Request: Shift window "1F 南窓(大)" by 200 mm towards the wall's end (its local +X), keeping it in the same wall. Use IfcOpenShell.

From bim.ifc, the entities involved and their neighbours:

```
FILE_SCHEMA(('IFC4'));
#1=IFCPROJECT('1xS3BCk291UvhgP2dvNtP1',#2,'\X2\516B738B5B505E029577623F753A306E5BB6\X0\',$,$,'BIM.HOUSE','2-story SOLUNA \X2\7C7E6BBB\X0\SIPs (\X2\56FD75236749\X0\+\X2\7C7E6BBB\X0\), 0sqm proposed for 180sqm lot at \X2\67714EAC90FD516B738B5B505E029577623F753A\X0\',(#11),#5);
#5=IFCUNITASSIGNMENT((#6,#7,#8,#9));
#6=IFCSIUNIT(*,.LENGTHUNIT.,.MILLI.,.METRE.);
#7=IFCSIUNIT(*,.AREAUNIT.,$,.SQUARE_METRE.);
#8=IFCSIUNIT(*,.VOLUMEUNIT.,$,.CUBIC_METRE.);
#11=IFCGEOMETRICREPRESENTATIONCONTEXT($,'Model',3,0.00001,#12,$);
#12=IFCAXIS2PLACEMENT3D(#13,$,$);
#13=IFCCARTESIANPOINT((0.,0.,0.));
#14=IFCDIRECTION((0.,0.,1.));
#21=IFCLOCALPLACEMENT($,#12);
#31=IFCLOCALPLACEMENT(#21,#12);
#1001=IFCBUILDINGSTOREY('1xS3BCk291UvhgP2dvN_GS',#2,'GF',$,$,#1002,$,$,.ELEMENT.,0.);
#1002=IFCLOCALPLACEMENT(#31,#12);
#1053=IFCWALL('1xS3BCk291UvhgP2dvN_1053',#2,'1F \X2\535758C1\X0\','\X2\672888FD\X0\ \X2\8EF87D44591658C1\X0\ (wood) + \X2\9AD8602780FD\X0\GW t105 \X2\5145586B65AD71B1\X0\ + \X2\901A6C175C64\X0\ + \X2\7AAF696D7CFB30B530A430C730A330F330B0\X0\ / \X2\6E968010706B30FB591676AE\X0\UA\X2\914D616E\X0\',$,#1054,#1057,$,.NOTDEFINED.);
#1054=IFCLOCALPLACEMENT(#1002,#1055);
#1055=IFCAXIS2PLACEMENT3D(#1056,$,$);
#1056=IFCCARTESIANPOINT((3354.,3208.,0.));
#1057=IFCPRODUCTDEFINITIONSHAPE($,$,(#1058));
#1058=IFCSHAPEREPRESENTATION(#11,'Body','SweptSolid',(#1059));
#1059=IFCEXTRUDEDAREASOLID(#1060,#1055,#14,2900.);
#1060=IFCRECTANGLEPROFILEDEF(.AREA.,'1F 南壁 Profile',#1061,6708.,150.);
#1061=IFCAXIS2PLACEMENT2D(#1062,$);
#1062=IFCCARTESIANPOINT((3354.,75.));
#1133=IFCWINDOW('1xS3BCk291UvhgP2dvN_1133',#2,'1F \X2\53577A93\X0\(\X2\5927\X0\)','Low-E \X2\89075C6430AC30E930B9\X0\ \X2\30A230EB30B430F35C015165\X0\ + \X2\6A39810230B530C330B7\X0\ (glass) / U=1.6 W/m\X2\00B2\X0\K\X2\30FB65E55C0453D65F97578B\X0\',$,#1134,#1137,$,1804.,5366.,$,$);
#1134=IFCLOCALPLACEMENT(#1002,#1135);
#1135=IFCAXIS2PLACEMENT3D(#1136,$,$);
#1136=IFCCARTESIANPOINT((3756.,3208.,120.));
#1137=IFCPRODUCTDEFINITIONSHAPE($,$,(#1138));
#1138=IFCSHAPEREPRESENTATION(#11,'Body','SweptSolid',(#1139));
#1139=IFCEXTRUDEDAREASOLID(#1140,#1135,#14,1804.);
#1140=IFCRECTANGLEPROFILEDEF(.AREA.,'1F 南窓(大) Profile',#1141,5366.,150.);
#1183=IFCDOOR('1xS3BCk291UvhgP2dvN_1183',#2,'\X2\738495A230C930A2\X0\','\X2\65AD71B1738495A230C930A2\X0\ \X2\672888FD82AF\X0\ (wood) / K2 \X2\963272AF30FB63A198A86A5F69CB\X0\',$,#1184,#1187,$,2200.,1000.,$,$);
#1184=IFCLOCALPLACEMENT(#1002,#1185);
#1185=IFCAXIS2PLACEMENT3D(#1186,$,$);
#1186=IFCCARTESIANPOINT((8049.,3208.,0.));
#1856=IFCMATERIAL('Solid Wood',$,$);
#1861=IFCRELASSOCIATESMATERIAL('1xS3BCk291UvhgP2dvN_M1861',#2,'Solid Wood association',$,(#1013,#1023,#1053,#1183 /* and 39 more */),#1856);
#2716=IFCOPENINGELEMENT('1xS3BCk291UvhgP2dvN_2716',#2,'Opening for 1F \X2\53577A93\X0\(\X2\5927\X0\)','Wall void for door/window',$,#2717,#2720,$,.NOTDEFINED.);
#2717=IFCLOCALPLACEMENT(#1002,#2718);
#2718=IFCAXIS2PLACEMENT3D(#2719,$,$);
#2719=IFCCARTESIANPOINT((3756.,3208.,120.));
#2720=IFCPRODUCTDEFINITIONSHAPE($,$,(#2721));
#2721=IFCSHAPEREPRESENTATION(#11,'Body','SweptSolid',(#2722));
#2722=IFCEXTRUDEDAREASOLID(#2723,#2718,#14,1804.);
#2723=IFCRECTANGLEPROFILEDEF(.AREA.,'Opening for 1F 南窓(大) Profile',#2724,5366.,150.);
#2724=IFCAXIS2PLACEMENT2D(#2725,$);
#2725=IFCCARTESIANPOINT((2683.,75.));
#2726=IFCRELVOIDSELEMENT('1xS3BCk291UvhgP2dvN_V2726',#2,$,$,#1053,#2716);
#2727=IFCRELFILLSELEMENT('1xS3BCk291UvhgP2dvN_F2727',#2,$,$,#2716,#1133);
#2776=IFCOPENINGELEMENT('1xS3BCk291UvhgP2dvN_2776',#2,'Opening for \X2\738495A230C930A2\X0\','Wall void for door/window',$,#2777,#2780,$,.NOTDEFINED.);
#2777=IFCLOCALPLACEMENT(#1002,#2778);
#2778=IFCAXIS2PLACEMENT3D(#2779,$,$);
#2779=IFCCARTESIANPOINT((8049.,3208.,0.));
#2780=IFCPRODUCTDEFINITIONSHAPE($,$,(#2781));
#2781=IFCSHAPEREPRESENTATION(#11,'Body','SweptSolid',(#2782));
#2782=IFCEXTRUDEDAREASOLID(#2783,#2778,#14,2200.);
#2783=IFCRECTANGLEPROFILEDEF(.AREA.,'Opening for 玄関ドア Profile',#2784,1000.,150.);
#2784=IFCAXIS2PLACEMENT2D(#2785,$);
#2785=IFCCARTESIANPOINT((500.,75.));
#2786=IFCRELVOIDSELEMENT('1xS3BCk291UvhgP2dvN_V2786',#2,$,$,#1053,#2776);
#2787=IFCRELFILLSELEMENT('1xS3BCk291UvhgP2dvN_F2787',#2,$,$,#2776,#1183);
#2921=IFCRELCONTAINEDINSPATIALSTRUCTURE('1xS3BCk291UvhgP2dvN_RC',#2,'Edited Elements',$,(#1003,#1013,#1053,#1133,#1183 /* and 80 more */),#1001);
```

```python
import ifcopenshell
import ifcopenshell.api.geometry
import ifcopenshell.util.placement
import ifcopenshell.util.unit

model = ifcopenshell.open("bim.ifc")
unit_scale = ifcopenshell.util.unit.calculate_unit_scale(model)

window = model.by_id(1133)
opening = window.FillsVoids[0].RelatingOpeningElement
wall = opening.VoidsElements[0].RelatingBuildingElement

wall_matrix = ifcopenshell.util.placement.get_local_placement(wall.ObjectPlacement)
shift = wall_matrix[:3, 0] * 0.2 / unit_scale
before = ifcopenshell.util.placement.get_local_placement(window.ObjectPlacement)[:3, 3].copy()

# The window is not placed relative to its opening, so move both.
for product in (opening, window):
    matrix = ifcopenshell.util.placement.get_local_placement(product.ObjectPlacement)
    matrix[:3, 3] += shift
    ifcopenshell.api.geometry.edit_object_placement(model, product=product, matrix=matrix, is_si=False)

after = ifcopenshell.util.placement.get_local_placement(window.ObjectPlacement)[:3, 3]
print("window moved by", (after - before).round(3) + 0.0)

model.write("bim_updated.ifc")
```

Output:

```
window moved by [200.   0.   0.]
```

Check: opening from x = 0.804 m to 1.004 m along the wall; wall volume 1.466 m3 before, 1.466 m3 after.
